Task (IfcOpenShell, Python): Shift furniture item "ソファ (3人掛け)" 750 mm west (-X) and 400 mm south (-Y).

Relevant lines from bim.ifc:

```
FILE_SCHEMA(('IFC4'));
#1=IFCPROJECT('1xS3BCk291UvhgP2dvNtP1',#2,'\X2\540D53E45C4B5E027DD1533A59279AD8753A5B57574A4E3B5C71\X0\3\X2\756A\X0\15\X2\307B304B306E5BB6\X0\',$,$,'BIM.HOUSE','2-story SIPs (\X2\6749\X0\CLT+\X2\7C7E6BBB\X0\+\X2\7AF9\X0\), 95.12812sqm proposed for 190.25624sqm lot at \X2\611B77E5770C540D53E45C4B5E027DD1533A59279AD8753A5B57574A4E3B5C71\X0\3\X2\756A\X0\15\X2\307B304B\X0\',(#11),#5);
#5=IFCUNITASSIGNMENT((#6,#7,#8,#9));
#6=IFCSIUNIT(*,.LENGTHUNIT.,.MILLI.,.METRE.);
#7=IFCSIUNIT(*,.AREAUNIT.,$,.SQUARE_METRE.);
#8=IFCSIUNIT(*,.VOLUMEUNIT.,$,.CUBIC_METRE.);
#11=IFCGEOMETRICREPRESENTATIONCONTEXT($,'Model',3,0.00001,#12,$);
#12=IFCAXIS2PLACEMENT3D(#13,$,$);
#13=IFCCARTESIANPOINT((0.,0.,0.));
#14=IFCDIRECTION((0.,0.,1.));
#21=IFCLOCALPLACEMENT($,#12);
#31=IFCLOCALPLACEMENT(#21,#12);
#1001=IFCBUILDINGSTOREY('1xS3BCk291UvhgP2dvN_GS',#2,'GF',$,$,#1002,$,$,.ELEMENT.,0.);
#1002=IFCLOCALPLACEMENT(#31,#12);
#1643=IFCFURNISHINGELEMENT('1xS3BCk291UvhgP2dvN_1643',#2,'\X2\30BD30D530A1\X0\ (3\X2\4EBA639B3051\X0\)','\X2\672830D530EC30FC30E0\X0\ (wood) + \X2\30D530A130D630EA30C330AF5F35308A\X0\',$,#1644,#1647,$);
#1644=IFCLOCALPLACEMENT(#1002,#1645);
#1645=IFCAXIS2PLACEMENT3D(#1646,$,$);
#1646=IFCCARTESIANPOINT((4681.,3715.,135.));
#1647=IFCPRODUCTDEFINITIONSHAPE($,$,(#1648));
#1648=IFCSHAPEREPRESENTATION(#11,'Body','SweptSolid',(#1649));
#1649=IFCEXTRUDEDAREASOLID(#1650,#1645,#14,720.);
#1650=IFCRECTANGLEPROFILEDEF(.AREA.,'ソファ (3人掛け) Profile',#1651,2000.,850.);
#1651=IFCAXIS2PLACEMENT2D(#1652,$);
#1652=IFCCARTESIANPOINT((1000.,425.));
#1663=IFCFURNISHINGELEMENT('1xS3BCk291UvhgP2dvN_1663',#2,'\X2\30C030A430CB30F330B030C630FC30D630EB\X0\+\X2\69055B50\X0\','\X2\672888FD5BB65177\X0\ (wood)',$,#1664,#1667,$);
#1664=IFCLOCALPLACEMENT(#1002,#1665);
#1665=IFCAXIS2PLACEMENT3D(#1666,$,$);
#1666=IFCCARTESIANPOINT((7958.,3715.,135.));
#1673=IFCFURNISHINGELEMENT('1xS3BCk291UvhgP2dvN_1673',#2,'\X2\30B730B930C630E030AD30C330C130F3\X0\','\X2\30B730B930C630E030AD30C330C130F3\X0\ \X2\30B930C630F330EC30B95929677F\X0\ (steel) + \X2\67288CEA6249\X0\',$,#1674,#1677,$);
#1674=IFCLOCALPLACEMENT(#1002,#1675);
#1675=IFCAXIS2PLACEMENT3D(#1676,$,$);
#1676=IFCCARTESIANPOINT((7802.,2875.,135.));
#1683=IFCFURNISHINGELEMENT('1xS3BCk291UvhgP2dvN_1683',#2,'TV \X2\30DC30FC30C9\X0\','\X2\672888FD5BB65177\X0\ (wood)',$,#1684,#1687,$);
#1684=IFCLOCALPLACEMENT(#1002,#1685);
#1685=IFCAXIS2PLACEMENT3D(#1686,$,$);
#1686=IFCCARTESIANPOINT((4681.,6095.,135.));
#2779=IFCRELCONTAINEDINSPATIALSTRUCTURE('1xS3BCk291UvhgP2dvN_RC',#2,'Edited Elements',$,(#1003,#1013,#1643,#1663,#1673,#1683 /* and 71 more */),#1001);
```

```python
import ifcopenshell
import ifcopenshell.api.geometry
import ifcopenshell.util.placement

model = ifcopenshell.open("bim.ifc")

item = model.by_guid("1xS3BCk291UvhgP2dvN_1643")
matrix = ifcopenshell.util.placement.get_local_placement(item.ObjectPlacement)
matrix[0, 3] -= 750.0
matrix[1, 3] -= 400.0
ifcopenshell.api.geometry.edit_object_placement(model, product=item, matrix=matrix, is_si=False)

print(ifcopenshell.util.placement.get_local_placement(item.ObjectPlacement).round(3) + 0.0)

model.write("bim_v2.ifc")
```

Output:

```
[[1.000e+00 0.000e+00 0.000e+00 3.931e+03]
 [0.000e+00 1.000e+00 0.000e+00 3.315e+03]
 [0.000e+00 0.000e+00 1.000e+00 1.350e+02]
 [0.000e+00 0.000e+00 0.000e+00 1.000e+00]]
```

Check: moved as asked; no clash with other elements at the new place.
